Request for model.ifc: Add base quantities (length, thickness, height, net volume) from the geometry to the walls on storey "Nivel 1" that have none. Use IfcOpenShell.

First a look at what the model holds.

```python
import ifcopenshell
import ifcopenshell.util.element
import ifcopenshell.util.unit

model = ifcopenshell.open("model.ifc")
print(model.schema)
for unit_type in ("LENGTHUNIT", "AREAUNIT", "VOLUMEUNIT"):
    print(unit_type, ifcopenshell.util.unit.calculate_unit_scale(model, unit_type))
storey = next(s for s in model.by_type("IfcBuildingStorey") if s.Name == "Nivel 1")
walls = [e for e in ifcopenshell.util.element.get_decomposition(storey) if e.is_a("IfcWall")]
for e in sorted(walls, key=lambda e: e.id()):
    print(e.id(), e.is_a(), e.Name, list(ifcopenshell.util.element.get_psets(e, qtos_only=True)), sep=" | ")
```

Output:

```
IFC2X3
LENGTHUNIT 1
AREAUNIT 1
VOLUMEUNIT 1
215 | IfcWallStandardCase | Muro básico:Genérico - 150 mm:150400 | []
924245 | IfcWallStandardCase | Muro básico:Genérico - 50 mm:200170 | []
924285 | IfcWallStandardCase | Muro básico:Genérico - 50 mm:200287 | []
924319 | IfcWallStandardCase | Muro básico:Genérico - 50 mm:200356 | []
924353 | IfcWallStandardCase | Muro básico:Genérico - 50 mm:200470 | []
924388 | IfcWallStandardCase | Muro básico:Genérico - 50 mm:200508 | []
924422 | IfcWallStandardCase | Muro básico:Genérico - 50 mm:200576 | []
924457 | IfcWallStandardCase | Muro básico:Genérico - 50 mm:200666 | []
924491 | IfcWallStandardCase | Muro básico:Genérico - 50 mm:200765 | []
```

```python
import ifcopenshell
import ifcopenshell.api.pset
import ifcopenshell.geom
import ifcopenshell.util.element
import ifcopenshell.util.shape
import ifcopenshell.util.unit

model = ifcopenshell.open("model.ifc")
unit_scale = ifcopenshell.util.unit.calculate_unit_scale(model)
volume_scale = ifcopenshell.util.unit.calculate_unit_scale(model, "VOLUMEUNIT")
settings = ifcopenshell.geom.settings()

storey = next(s for s in model.by_type("IfcBuildingStorey") if s.Name == "Nivel 1")
walls = [e for e in ifcopenshell.util.element.get_decomposition(storey) if e.is_a("IfcWall")]

for e in sorted(walls, key=lambda e: e.id()):
    if ifcopenshell.util.element.get_psets(e, qtos_only=True, should_inherit=False):
        continue
    # Geometry comes back in metres, in the element's own axes.
    shape = ifcopenshell.geom.create_shape(settings, e)
    values = {
        "Length": ifcopenshell.util.shape.get_x(shape.geometry) / unit_scale,
        "Width": ifcopenshell.util.shape.get_y(shape.geometry) / unit_scale,
        "Height": ifcopenshell.util.shape.get_z(shape.geometry) / unit_scale,
        "NetVolume": ifcopenshell.util.shape.get_volume(shape.geometry) / volume_scale,
    }
    qto = ifcopenshell.api.pset.add_qto(model, product=e, name="BaseQuantities")
    ifcopenshell.api.pset.edit_qto(model, qto=qto, properties=values)
    print(e.id(), {k: round(v, 3) for k, v in values.items()})

model.write("model_rev.ifc")
```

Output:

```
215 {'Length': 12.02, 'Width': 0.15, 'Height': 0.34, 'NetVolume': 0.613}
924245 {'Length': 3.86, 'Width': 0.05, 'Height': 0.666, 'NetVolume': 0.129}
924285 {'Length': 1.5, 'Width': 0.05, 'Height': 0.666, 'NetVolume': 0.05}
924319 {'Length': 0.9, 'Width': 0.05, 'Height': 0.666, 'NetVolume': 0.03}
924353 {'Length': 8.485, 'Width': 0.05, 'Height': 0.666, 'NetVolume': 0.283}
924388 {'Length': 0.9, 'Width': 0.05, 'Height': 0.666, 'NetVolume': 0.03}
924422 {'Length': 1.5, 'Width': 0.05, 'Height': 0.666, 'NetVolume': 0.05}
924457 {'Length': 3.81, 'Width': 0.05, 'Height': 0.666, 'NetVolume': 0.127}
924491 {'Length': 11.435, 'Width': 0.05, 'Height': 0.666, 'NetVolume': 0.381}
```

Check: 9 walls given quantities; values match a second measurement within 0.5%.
